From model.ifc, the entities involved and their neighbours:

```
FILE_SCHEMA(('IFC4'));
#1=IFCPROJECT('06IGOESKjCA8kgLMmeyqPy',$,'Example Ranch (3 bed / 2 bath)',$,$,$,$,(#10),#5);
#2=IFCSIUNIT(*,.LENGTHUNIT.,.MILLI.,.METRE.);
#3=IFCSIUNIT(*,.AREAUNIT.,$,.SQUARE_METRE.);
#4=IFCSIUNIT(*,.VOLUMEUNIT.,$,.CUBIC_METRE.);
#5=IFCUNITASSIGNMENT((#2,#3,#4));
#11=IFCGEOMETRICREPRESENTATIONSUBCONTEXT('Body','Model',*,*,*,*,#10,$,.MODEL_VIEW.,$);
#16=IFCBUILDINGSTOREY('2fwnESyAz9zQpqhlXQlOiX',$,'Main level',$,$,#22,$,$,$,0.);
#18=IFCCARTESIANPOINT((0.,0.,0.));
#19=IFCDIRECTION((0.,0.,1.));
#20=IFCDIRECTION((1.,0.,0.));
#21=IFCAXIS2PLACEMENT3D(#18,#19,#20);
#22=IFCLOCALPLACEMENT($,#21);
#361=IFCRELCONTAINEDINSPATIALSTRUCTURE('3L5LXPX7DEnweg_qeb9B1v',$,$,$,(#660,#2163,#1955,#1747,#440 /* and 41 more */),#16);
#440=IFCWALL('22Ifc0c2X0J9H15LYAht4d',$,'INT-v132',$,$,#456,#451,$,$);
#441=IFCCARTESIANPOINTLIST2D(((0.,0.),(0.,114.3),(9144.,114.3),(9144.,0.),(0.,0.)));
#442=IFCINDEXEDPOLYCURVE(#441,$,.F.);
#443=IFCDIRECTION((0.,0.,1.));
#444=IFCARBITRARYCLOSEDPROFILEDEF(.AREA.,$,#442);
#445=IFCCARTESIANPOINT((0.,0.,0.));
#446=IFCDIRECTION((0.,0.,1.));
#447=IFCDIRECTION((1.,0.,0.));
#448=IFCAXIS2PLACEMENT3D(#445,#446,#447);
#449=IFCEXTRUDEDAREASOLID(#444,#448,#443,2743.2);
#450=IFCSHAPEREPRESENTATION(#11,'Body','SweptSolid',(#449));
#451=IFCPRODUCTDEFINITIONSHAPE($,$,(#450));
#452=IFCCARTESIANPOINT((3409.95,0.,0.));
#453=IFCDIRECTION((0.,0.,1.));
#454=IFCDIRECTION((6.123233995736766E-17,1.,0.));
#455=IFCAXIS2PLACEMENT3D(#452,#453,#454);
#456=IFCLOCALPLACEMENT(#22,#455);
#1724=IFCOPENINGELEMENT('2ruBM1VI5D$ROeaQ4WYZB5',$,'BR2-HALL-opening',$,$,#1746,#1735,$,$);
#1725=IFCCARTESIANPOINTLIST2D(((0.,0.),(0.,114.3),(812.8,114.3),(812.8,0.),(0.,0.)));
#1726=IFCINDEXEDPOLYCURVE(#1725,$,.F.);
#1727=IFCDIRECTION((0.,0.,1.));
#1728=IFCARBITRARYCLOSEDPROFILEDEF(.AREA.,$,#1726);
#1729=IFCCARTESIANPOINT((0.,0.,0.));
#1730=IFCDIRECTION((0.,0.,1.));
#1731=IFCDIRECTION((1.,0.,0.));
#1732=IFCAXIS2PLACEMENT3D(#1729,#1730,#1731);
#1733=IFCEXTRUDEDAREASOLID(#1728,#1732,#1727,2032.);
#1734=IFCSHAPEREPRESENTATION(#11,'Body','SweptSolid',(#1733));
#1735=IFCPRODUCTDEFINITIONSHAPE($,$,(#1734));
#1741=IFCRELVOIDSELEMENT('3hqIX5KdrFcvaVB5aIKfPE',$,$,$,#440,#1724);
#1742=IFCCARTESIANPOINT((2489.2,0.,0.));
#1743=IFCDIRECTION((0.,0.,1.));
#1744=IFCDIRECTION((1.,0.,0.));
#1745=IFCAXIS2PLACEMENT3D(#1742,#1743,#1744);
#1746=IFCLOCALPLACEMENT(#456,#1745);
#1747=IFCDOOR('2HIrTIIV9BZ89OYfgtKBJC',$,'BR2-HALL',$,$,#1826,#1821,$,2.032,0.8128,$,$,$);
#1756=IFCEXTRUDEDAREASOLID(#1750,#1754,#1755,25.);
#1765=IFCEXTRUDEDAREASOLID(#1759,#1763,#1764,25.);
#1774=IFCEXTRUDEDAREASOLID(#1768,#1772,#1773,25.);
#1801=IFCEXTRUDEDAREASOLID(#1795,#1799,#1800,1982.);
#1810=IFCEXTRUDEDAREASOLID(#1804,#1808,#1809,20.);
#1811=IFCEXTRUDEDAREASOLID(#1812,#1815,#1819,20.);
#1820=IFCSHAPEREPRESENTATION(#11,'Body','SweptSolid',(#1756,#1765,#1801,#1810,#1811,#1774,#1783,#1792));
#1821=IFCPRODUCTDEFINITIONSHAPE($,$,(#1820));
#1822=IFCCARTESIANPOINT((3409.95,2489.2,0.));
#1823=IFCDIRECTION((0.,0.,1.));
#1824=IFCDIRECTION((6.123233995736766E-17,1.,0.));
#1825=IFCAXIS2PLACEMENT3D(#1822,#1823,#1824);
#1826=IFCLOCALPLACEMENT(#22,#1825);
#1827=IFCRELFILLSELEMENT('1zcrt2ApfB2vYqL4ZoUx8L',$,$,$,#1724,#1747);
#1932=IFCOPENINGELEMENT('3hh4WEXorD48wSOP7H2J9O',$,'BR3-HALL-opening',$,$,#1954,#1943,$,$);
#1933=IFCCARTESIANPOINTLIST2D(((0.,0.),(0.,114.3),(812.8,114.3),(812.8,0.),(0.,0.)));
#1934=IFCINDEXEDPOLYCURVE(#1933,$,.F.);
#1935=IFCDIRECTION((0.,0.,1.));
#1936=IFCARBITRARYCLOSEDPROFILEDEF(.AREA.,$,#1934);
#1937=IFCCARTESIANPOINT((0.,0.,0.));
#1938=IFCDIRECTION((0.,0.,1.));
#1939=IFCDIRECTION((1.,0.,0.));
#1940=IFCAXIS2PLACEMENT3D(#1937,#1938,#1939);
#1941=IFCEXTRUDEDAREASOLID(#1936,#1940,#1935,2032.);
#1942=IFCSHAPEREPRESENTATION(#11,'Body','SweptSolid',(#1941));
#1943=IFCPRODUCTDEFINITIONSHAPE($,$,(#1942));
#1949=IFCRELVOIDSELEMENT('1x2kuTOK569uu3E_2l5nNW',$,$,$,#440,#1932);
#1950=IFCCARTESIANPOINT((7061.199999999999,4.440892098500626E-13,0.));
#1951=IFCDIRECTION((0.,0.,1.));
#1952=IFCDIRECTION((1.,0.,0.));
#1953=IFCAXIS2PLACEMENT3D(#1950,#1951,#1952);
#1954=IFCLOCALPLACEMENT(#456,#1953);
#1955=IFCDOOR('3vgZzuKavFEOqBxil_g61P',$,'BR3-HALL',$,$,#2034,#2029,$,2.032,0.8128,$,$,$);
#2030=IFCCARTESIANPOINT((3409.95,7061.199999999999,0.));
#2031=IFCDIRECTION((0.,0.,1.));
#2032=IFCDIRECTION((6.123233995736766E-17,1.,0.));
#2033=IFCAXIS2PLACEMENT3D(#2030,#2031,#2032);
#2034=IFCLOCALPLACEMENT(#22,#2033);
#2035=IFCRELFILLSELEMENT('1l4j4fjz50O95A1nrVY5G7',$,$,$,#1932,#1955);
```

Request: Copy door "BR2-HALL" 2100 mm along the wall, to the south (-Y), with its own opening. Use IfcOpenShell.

```python
import ifcopenshell
import ifcopenshell.api.feature
import ifcopenshell.api.geometry
import ifcopenshell.api.root
import ifcopenshell.geom
import ifcopenshell.util.element
import ifcopenshell.util.placement
import ifcopenshell.util.shape
import ifcopenshell.util.unit

model = ifcopenshell.open("model.ifc")
unit_scale = ifcopenshell.util.unit.calculate_unit_scale(model)
settings = ifcopenshell.geom.settings()


def volume(element):
    """Net volume in cubic metres, openings subtracted."""
    shape = ifcopenshell.geom.create_shape(settings, element)
    return ifcopenshell.util.shape.get_volume(shape.geometry)


door = model.by_id(1747)
opening = door.FillsVoids[0].RelatingOpeningElement
wall = opening.VoidsElements[0].RelatingBuildingElement
before = volume(wall)
shift = ifcopenshell.util.placement.get_local_placement(wall.ObjectPlacement)[:3, 0] * -2.1 / unit_scale

# copy_class copies the void relationship, type, container and properties, but no geometry.
new_opening = ifcopenshell.api.root.copy_class(model, product=opening)
new_opening.Representation = ifcopenshell.util.element.copy_deep(
    model, opening.Representation, exclude=["IfcGeometricRepresentationContext", "IfcRepresentationMap"]
)
new_door = ifcopenshell.api.root.copy_class(model, product=door)
new_door.Representation = ifcopenshell.util.element.copy_deep(
    model, door.Representation, exclude=["IfcGeometricRepresentationContext", "IfcRepresentationMap"]
)
ifcopenshell.api.feature.add_filling(model, opening=new_opening, element=new_door)

for old, new in ((opening, new_opening), (door, new_door)):
    matrix = ifcopenshell.util.placement.get_local_placement(old.ObjectPlacement)
    matrix[:3, 3] += shift
    ifcopenshell.api.geometry.edit_object_placement(model, product=new, matrix=matrix, is_si=False)

after = volume(wall)

print(f"wall volume {before:.3f} -> {after:.3f} m3")

model.write("model_rev.ifc")
```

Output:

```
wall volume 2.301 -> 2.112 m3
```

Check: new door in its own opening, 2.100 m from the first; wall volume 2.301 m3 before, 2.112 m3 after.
